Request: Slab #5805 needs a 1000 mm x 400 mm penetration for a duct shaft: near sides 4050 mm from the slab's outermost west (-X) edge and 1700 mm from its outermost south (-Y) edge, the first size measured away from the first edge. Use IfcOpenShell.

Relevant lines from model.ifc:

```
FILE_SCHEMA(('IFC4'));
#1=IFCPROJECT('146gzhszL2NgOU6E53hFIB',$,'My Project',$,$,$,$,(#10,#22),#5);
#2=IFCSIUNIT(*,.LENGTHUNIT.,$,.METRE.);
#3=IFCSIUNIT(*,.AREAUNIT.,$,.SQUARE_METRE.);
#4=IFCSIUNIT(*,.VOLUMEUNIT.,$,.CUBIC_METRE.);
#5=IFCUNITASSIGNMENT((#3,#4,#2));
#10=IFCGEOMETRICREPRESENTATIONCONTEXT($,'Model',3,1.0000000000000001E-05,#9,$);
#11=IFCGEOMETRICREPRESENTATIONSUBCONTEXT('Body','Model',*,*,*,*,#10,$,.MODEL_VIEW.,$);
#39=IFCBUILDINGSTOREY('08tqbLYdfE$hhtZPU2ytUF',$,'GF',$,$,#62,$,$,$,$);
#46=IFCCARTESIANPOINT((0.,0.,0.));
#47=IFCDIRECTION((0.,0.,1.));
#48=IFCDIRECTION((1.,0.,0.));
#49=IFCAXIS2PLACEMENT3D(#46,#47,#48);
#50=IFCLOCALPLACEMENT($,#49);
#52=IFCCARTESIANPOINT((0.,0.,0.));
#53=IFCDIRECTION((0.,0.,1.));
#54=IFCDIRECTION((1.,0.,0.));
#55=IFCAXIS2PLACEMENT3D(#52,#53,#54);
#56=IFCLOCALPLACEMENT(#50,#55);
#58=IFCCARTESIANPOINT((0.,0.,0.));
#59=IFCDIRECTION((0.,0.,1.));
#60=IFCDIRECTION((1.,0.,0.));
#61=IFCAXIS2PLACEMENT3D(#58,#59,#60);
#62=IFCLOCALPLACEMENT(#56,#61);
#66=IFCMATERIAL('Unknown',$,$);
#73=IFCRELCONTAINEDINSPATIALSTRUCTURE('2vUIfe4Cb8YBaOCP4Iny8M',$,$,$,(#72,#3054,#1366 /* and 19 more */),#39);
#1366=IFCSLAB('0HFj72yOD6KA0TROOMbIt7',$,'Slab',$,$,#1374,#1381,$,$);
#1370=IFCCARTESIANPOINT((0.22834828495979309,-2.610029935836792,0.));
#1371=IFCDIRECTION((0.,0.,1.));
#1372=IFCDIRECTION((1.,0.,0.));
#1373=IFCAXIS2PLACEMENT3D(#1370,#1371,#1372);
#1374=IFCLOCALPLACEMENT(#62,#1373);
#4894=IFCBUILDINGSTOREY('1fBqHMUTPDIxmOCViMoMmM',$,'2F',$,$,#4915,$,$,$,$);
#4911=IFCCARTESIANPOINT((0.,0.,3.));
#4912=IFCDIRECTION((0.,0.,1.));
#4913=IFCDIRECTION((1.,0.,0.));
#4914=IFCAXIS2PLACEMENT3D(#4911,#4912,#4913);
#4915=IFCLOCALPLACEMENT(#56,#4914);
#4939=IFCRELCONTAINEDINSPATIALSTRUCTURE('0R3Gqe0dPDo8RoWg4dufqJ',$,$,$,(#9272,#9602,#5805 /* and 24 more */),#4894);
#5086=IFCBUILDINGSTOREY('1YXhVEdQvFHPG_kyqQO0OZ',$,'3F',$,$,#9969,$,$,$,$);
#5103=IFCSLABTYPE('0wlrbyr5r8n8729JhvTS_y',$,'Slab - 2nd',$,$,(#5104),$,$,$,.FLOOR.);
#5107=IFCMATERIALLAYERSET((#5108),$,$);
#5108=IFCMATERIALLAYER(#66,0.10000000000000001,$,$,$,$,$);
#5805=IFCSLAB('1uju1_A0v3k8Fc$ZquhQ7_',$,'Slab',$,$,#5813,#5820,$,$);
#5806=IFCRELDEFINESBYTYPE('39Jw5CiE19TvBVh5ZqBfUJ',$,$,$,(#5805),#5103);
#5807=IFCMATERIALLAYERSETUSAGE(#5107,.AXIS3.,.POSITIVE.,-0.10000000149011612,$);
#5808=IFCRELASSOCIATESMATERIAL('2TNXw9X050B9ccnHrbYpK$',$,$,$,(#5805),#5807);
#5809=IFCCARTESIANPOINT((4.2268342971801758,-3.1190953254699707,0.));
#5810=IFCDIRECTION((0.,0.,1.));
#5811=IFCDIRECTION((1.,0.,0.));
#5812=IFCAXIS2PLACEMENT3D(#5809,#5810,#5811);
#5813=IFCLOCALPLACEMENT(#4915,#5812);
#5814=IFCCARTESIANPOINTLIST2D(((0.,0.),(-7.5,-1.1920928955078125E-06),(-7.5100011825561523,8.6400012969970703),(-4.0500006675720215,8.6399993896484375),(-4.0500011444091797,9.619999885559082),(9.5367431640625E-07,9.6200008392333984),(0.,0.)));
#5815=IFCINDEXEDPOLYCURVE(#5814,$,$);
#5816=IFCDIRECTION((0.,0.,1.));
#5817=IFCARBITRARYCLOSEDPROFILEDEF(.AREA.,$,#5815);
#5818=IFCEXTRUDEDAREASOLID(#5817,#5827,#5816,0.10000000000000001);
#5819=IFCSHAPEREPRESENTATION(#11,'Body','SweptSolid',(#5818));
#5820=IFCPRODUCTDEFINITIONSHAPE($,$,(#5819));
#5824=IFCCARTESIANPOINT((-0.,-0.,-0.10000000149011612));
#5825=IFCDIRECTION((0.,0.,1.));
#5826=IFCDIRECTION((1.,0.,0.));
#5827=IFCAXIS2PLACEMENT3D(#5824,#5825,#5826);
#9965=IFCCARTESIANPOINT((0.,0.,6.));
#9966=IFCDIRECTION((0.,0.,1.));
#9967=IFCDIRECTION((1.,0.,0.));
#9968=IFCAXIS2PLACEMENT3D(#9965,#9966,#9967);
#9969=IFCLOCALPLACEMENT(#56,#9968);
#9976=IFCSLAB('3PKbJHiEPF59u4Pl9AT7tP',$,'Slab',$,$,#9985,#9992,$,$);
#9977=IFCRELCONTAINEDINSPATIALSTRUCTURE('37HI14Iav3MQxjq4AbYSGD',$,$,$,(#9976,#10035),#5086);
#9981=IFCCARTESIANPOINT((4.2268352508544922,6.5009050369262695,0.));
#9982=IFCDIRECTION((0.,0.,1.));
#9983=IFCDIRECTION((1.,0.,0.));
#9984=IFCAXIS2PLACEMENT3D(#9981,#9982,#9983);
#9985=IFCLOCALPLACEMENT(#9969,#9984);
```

```python
import numpy as np
import ifcopenshell
import ifcopenshell.api.feature
import ifcopenshell.api.geometry
import ifcopenshell.api.root
import ifcopenshell.geom
import ifcopenshell.util.placement
import ifcopenshell.util.representation
import ifcopenshell.util.shape
import ifcopenshell.util.unit

model = ifcopenshell.open("model.ifc")
unit_scale = ifcopenshell.util.unit.calculate_unit_scale(model)
settings = ifcopenshell.geom.settings()


def volume(element):
    """Net volume in cubic metres, openings subtracted."""
    shape = ifcopenshell.geom.create_shape(settings, element)
    return ifcopenshell.util.shape.get_volume(shape.geometry)


slab = model.by_guid("1uju1_A0v3k8Fc$ZquhQ7_")
before = volume(slab)

# Extent in the slab's own axes, in metres. The edges named are its -X and -Y sides.
slab_shape = ifcopenshell.geom.create_shape(settings, slab)
vertices = ifcopenshell.util.shape.get_vertices(slab_shape.geometry)
x_min, y_min, bottom = vertices.min(axis=0)
top = vertices[:, 2].max()

opening = ifcopenshell.api.root.create_entity(model, ifc_class="IfcOpeningElement", name="Duct shaft opening", predefined_type="OPENING")
context = ifcopenshell.util.representation.get_context(model, "Model", "Body", "MODEL_VIEW")
width, depth = 1, 0.4
outline = [(0.0, 0.0), (width, 0.0), (width, depth), (0.0, depth), (0.0, 0.0)]
# Overshoot both faces by 50 mm so the cut is clean.
shape = ifcopenshell.api.geometry.add_slab_representation(
    model, context=context, depth=top - bottom + 0.1, polyline=outline
)
ifcopenshell.api.geometry.assign_representation(model, product=opening, representation=shape)

matrix = ifcopenshell.util.placement.get_local_placement(slab.ObjectPlacement)
matrix[:, 3] = matrix @ np.append(np.array([x_min + 4.05, y_min + 1.7, bottom - 0.05]) / unit_scale, 1.0)
ifcopenshell.api.geometry.edit_object_placement(model, product=opening, matrix=matrix, is_si=False)
ifcopenshell.api.feature.add_feature(model, feature=opening, element=slab)

after = volume(slab)

print(f"slab volume {before:.3f} -> {after:.3f} m3")

model.write("model_v2.ifc")
```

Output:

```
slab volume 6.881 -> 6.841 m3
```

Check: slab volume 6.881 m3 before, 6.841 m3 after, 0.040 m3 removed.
